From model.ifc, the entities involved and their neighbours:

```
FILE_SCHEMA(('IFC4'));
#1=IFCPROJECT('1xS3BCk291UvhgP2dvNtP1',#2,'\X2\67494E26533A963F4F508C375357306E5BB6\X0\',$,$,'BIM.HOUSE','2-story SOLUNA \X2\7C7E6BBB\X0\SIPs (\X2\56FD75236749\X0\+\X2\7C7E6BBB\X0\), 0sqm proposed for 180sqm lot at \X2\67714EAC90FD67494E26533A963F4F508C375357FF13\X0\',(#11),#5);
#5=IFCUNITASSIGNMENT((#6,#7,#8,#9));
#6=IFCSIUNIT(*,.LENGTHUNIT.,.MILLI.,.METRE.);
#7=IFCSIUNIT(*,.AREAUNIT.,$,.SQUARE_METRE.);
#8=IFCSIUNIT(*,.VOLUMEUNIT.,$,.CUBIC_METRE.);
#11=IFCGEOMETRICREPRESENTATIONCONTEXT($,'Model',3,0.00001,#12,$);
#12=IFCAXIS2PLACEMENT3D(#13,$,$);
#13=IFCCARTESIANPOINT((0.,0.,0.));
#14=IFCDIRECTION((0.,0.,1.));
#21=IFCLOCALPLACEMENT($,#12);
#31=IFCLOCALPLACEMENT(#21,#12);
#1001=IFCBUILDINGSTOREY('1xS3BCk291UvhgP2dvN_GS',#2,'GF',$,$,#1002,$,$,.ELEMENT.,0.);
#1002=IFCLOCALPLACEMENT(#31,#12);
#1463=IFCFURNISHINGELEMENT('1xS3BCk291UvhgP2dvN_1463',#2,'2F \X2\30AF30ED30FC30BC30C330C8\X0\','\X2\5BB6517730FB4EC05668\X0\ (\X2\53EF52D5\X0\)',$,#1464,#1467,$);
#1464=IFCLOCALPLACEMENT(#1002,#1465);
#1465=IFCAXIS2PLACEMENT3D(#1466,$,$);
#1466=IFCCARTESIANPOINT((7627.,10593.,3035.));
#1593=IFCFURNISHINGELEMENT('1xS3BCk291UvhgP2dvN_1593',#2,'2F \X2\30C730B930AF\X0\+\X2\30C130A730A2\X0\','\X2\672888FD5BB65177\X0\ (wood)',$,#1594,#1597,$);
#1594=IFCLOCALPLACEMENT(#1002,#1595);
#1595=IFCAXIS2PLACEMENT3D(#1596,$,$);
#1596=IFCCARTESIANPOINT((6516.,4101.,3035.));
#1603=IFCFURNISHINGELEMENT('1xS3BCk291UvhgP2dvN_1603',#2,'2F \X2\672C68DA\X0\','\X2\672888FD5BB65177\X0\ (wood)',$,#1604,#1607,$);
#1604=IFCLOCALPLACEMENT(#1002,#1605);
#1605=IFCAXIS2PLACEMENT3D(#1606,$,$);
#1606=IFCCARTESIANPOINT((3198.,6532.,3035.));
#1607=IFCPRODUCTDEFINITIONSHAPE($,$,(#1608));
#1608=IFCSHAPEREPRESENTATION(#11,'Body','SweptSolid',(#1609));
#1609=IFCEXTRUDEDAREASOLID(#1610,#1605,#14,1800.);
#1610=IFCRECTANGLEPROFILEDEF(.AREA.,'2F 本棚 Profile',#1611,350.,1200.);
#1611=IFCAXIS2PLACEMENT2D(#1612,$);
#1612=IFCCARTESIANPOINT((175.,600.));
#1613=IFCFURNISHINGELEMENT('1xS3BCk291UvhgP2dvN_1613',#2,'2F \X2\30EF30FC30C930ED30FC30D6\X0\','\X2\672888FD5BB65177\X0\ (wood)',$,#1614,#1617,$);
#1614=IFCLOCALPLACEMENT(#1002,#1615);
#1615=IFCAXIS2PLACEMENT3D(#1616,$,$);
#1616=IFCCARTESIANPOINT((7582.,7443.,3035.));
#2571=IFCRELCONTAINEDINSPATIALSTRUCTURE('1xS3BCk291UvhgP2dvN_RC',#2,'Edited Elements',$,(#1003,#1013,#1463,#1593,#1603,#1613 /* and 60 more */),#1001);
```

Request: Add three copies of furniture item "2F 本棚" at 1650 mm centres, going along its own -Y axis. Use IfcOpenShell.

```python
import ifcopenshell
import ifcopenshell.api.geometry
import ifcopenshell.api.root
import ifcopenshell.util.element
import ifcopenshell.util.placement

model = ifcopenshell.open("model.ifc")


def reuse_history(source, copy):
    """copy_class also copies each property set's owner history, people and application; keep the originals."""
    for rel in copy.IsDefinedBy:
        if rel.is_a("IfcRelDefinesByProperties") and (history := rel.RelatingPropertyDefinition.OwnerHistory):
            rel.RelatingPropertyDefinition.OwnerHistory = source.OwnerHistory
            ifcopenshell.util.element.remove_deep2(model, history)


source = model.by_id(1603)
base = ifcopenshell.util.placement.get_local_placement(source.ObjectPlacement)
step = -base[:3, 1] * 1650.0

for i in range(1, 4):
    copy = ifcopenshell.api.root.copy_class(model, product=source)
    copy.Representation = ifcopenshell.util.element.copy_deep(
        model, source.Representation, exclude=["IfcGeometricRepresentationContext", "IfcRepresentationMap"]
    )
    reuse_history(source, copy)
    matrix = base.copy()
    matrix[:3, 3] += i * step
    print("added at", matrix[:3, 3].round(3) + 0.0)
    ifcopenshell.api.geometry.edit_object_placement(model, product=copy, matrix=matrix, is_si=False)

model.write("model_v2.ifc")
```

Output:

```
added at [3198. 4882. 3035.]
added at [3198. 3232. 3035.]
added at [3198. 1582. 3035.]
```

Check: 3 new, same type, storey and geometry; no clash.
